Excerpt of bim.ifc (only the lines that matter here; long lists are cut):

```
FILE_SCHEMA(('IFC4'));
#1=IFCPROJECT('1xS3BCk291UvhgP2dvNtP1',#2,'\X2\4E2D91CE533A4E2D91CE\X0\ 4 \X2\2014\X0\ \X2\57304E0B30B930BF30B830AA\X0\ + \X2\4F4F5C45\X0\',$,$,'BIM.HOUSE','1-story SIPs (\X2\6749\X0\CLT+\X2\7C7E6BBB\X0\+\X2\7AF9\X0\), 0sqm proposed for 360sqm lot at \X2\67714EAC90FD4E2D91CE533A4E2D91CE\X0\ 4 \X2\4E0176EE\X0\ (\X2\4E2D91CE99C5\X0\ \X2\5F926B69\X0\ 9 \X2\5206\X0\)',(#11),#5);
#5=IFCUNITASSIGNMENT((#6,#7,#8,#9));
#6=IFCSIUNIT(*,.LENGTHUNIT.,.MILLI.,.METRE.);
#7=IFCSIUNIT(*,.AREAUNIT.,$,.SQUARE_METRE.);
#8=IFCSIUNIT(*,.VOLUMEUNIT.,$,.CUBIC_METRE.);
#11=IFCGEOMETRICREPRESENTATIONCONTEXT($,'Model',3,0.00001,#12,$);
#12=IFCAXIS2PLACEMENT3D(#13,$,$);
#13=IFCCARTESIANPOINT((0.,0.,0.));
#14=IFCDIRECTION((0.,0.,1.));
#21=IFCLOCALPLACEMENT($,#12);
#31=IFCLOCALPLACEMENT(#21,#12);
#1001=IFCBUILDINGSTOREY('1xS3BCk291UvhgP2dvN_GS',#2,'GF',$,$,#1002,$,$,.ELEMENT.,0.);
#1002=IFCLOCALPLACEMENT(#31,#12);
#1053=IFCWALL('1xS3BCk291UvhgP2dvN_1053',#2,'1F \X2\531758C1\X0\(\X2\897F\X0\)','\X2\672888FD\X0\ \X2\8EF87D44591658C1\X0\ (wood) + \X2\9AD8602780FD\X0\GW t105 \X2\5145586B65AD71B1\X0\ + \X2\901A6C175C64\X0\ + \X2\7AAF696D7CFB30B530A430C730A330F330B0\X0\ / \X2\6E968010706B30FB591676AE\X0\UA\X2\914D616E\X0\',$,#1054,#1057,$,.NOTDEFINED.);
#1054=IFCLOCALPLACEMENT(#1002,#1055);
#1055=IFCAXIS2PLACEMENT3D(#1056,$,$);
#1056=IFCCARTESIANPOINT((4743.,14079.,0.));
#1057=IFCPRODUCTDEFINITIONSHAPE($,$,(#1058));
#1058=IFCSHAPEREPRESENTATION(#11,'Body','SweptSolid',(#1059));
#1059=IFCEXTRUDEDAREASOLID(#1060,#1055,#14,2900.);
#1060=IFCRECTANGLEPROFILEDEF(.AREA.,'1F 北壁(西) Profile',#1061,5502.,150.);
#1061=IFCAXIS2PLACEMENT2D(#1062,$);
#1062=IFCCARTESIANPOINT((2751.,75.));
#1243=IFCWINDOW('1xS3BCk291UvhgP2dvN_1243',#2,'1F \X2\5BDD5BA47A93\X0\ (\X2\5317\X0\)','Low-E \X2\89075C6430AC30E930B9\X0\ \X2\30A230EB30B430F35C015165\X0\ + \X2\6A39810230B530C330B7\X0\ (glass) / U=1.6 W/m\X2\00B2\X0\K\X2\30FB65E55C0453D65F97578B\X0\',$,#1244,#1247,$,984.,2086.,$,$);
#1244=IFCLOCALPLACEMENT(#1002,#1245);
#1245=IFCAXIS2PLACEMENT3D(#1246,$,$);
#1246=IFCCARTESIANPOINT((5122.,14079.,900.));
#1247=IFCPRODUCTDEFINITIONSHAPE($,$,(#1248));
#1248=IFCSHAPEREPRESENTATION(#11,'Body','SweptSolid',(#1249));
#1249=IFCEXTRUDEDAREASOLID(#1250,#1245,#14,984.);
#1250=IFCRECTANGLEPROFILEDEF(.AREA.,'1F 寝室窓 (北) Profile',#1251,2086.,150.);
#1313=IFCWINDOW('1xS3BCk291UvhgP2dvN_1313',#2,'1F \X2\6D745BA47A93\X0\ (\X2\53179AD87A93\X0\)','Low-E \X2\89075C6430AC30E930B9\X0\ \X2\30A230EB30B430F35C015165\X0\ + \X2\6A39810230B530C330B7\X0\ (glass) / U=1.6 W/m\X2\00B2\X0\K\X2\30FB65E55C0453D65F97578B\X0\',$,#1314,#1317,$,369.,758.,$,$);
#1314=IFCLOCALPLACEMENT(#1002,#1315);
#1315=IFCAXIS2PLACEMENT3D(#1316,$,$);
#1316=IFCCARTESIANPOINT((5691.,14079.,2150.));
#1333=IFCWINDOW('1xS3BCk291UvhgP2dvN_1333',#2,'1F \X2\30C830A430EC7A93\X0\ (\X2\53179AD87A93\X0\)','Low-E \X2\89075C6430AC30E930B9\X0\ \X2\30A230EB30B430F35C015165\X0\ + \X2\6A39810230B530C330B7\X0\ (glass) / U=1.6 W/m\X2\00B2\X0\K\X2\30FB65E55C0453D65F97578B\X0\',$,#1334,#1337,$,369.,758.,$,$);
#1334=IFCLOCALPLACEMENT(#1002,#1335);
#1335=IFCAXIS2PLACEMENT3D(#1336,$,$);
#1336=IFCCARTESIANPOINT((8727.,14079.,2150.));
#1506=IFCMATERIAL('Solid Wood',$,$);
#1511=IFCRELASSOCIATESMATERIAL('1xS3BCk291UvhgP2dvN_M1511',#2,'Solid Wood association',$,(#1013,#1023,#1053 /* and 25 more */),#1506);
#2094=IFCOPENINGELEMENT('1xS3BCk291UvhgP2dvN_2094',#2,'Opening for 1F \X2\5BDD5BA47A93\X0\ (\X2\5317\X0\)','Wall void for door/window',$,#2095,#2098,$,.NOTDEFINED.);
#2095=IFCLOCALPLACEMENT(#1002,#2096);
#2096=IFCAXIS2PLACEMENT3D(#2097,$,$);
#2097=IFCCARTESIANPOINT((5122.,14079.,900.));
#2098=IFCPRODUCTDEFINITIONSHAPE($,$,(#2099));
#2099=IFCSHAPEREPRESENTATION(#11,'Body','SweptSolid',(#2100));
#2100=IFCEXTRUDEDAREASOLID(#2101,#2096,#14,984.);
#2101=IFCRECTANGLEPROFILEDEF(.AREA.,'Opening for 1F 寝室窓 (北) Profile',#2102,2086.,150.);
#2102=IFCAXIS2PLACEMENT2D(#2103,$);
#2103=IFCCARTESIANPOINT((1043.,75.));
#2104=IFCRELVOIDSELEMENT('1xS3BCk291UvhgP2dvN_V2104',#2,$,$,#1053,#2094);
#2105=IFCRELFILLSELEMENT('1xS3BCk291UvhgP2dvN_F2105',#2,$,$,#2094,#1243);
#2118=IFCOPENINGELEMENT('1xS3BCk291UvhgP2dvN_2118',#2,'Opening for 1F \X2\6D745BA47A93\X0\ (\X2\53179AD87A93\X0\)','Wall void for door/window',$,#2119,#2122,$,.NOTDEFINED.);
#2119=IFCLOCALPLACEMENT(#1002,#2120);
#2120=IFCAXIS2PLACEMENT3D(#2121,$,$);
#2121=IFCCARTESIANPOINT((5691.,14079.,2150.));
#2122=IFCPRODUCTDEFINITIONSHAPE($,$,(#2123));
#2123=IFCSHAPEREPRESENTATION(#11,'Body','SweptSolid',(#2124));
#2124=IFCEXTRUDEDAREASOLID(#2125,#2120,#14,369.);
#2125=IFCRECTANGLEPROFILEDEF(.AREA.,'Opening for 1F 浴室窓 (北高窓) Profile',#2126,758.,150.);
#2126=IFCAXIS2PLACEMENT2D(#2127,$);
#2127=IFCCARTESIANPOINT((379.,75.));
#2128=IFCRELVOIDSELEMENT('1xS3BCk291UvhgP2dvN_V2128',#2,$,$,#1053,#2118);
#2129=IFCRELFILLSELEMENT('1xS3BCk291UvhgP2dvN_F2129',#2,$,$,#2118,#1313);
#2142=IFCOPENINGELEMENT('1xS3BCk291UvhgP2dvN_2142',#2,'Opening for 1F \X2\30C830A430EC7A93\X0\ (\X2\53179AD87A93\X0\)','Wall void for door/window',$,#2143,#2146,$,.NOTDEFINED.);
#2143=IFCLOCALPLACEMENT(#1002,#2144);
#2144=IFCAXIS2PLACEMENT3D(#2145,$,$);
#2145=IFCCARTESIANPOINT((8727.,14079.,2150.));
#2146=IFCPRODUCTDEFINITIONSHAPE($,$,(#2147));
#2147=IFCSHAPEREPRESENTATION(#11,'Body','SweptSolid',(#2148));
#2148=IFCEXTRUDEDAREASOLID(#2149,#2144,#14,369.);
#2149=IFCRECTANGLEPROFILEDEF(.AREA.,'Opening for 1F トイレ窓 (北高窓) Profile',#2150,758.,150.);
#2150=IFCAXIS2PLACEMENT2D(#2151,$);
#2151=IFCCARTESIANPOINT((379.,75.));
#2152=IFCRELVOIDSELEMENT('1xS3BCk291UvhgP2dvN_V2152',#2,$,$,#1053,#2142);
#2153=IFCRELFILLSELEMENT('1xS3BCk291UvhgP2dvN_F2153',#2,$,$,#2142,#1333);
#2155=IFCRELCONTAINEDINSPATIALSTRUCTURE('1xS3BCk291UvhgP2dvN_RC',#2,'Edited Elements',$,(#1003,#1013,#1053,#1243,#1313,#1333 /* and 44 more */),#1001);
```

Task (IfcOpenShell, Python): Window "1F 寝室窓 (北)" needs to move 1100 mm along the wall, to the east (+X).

```python
import ifcopenshell
import ifcopenshell.api.geometry
import ifcopenshell.util.placement

model = ifcopenshell.open("bim.ifc")

window = model.by_guid("1xS3BCk291UvhgP2dvN_1243")
opening = window.FillsVoids[0].RelatingOpeningElement
wall = opening.VoidsElements[0].RelatingBuildingElement

wall_matrix = ifcopenshell.util.placement.get_local_placement(wall.ObjectPlacement)
shift = wall_matrix[:3, 0] * 1100.0
before = ifcopenshell.util.placement.get_local_placement(window.ObjectPlacement)[:3, 3].copy()

# The window is not placed relative to its opening, so move both.
for product in (opening, window):
    matrix = ifcopenshell.util.placement.get_local_placement(product.ObjectPlacement)
    matrix[:3, 3] += shift
    ifcopenshell.api.geometry.edit_object_placement(model, product=product, matrix=matrix, is_si=False)

after = ifcopenshell.util.placement.get_local_placement(window.ObjectPlacement)[:3, 3]
print("window moved by", (after - before).round(3) + 0.0)

model.write("bim_updated.ifc")
```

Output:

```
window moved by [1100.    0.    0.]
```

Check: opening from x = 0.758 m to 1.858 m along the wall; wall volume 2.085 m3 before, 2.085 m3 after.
